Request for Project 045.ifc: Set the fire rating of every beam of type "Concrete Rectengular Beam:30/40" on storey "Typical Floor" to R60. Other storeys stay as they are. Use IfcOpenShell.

First a look at what the model holds.

```python
import ifcopenshell
import ifcopenshell.util.element

model = ifcopenshell.open("Project 045.ifc")
print(model.schema)
storey = next(s for s in model.by_type("IfcBuildingStorey") if s.Name == "Typical Floor")
beams = [e for e in ifcopenshell.util.element.get_decomposition(storey) if e.is_a("IfcBeam")]
seen = {}
for e in beams:
    element_type = ifcopenshell.util.element.get_type(e)
    key = (element_type.Name if element_type != e and element_type else None, ifcopenshell.util.element.get_pset(e, "Pset_BeamCommon", "FireRating"))
    seen[key] = seen.get(key, 0) + 1
for (name, value), count in sorted(seen.items(), key=str):
    print(count, "x", name, "|", value)
```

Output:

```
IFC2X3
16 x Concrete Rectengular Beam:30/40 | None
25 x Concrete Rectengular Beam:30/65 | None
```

```python
import ifcopenshell
import ifcopenshell.api.pset
import ifcopenshell.util.element

model = ifcopenshell.open("Project 045.ifc")

storey = next(s for s in model.by_type("IfcBuildingStorey") if s.Name == "Typical Floor")
beams = [e for e in ifcopenshell.util.element.get_decomposition(storey) if e.is_a("IfcBeam")]

count = 0
for e in beams:
    element_type = ifcopenshell.util.element.get_type(e)
    if element_type in (None, e) or element_type.Name != "Concrete Rectengular Beam:30/40":
        continue
    # add_pset returns the element's existing set when there is one.
    pset = ifcopenshell.api.pset.add_pset(model, product=e, name="Pset_BeamCommon")
    ifcopenshell.api.pset.edit_pset(model, pset=pset, properties={"FireRating": "R60"})
    count += 1

print(count, "beams updated")

model.write("Project 045-out.ifc")
```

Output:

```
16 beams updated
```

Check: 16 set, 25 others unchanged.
